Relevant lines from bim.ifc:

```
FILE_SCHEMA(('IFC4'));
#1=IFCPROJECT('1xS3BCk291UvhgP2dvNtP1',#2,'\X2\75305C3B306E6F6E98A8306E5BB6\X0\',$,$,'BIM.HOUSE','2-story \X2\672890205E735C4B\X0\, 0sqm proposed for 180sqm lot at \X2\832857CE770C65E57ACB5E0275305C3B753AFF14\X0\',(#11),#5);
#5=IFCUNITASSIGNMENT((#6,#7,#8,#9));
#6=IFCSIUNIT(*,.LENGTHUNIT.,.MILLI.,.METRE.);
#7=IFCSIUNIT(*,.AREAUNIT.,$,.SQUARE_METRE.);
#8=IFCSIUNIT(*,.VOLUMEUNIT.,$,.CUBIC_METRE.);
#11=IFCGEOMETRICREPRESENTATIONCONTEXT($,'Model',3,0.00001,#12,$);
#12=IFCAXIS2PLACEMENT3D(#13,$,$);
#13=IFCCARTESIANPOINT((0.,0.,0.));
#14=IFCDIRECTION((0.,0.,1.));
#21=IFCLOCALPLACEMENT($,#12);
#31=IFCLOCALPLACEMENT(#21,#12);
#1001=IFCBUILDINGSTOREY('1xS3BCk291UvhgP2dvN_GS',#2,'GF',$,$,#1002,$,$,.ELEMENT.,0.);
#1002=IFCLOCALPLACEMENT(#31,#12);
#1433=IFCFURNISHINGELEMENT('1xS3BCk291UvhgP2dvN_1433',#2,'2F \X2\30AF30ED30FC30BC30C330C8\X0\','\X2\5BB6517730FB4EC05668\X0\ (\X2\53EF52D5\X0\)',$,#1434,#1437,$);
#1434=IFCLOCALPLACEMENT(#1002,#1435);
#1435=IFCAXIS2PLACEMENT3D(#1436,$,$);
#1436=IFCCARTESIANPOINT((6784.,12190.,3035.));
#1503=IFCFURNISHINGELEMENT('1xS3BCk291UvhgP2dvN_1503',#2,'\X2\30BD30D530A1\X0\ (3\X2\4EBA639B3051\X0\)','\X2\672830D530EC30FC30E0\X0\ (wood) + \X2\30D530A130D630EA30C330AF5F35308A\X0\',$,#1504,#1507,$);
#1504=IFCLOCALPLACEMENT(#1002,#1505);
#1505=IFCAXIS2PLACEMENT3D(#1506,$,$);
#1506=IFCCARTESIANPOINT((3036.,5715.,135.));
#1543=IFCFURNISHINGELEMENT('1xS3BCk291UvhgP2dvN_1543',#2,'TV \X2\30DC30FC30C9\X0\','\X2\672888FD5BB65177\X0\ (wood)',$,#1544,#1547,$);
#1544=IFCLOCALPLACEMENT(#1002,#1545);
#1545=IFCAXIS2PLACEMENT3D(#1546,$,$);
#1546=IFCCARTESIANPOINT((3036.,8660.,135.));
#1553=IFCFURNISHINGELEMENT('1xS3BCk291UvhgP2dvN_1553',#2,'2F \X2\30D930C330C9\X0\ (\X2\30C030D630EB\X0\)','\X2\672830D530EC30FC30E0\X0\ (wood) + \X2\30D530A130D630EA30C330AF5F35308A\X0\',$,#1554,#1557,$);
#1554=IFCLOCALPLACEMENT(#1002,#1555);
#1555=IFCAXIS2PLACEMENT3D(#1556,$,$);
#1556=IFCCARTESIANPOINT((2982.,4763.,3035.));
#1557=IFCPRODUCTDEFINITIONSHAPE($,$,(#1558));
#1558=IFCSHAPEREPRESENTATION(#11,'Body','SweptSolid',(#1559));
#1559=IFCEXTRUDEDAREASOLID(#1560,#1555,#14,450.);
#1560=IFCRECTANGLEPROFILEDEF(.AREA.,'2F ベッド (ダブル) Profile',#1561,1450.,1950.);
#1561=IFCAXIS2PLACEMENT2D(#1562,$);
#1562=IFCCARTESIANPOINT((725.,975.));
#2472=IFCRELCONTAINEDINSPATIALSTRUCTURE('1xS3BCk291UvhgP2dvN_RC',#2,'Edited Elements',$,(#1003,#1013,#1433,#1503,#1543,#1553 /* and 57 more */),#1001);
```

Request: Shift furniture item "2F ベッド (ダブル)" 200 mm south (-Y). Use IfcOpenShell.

```python
import ifcopenshell
import ifcopenshell.api.geometry
import ifcopenshell.util.placement
import ifcopenshell.util.unit

model = ifcopenshell.open("bim.ifc")
unit_scale = ifcopenshell.util.unit.calculate_unit_scale(model)

item = model.by_guid("1xS3BCk291UvhgP2dvN_1553")
matrix = ifcopenshell.util.placement.get_local_placement(item.ObjectPlacement)
matrix[1, 3] -= 0.2 / unit_scale
ifcopenshell.api.geometry.edit_object_placement(model, product=item, matrix=matrix, is_si=False)

print(ifcopenshell.util.placement.get_local_placement(item.ObjectPlacement).round(3) + 0.0)

model.write("bim_v2.ifc")
```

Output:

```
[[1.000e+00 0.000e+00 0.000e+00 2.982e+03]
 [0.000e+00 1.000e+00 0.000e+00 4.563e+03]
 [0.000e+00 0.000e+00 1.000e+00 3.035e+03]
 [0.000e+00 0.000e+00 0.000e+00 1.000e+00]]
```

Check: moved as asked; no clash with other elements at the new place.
